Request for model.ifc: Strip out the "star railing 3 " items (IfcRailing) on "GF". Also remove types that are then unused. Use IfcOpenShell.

First a look at what the model holds.

```python
import ifcopenshell
import ifcopenshell.util.element

model = ifcopenshell.open("model.ifc")
print(model.schema)
storey = next(s for s in model.by_type("IfcBuildingStorey") if s.Name == "GF")
railings = [e for e in ifcopenshell.util.element.get_decomposition(storey) if e.is_a("IfcRailing")]
seen = {}
for e in railings:
    element_type = ifcopenshell.util.element.get_type(e)
    name = element_type.Name if element_type not in (None, e) else None
    seen[name] = seen.get(name, 0) + 1
for name, count in sorted(seen.items(), key=str):
    print(count, "x", name)
```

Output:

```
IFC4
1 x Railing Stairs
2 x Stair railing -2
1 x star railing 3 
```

```python
import ifcopenshell
import ifcopenshell.api.root
import ifcopenshell.util.element

model = ifcopenshell.open("model.ifc")

storey = next(s for s in model.by_type("IfcBuildingStorey") if s.Name == "GF")
railings = [e for e in ifcopenshell.util.element.get_decomposition(storey) if e.is_a("IfcRailing")]
targets = [e for e in railings if (t := ifcopenshell.util.element.get_type(e)) not in (None, e) and t.Name == "star railing 3 "]
types = {ifcopenshell.util.element.get_type(e) for e in targets} - {None, *targets}

for e in targets:
    ifcopenshell.api.root.remove_product(model, product=e)
print(len(targets), "removed")

unused = [t for t in types if not ifcopenshell.util.element.get_types(t)]
for t in unused:
    ifcopenshell.api.root.remove_product(model, product=t)
print(len(unused), "unused types removed")

model.write("model_v2.ifc")
```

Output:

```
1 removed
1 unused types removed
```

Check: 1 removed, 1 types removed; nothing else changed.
